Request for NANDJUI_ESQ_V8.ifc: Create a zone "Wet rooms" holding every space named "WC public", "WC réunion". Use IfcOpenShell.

First a look at what the model holds.

```python
import ifcopenshell

model = ifcopenshell.open("NANDJUI_ESQ_V8.ifc")
print(model.schema)
seen = {}
for space in model.by_type("IfcSpace"):
    seen[space.LongName] = seen.get(space.LongName, 0) + 1
for name, count in sorted(seen.items(), key=str):
    print(count, "x", name)
print("zones:", [z.Name for z in model.by_type("IfcZone")][:20])
```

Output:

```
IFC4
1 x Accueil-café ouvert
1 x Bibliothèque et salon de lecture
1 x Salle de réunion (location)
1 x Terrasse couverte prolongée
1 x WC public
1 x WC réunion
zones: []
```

```python
import ifcopenshell
import ifcopenshell.api.group
import ifcopenshell.api.root

model = ifcopenshell.open("NANDJUI_ESQ_V8.ifc")

names = {"WC public", "WC réunion"}
spaces = [s for s in model.by_type("IfcSpace") if s.LongName in names]

zone = ifcopenshell.api.root.create_entity(model, ifc_class="IfcZone", name="Wet rooms")
ifcopenshell.api.group.assign_group(model, products=spaces, group=zone)
print(len(spaces), "spaces in", zone.Name)

model.write("NANDJUI_ESQ_V8_v2.ifc")
```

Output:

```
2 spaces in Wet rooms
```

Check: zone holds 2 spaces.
